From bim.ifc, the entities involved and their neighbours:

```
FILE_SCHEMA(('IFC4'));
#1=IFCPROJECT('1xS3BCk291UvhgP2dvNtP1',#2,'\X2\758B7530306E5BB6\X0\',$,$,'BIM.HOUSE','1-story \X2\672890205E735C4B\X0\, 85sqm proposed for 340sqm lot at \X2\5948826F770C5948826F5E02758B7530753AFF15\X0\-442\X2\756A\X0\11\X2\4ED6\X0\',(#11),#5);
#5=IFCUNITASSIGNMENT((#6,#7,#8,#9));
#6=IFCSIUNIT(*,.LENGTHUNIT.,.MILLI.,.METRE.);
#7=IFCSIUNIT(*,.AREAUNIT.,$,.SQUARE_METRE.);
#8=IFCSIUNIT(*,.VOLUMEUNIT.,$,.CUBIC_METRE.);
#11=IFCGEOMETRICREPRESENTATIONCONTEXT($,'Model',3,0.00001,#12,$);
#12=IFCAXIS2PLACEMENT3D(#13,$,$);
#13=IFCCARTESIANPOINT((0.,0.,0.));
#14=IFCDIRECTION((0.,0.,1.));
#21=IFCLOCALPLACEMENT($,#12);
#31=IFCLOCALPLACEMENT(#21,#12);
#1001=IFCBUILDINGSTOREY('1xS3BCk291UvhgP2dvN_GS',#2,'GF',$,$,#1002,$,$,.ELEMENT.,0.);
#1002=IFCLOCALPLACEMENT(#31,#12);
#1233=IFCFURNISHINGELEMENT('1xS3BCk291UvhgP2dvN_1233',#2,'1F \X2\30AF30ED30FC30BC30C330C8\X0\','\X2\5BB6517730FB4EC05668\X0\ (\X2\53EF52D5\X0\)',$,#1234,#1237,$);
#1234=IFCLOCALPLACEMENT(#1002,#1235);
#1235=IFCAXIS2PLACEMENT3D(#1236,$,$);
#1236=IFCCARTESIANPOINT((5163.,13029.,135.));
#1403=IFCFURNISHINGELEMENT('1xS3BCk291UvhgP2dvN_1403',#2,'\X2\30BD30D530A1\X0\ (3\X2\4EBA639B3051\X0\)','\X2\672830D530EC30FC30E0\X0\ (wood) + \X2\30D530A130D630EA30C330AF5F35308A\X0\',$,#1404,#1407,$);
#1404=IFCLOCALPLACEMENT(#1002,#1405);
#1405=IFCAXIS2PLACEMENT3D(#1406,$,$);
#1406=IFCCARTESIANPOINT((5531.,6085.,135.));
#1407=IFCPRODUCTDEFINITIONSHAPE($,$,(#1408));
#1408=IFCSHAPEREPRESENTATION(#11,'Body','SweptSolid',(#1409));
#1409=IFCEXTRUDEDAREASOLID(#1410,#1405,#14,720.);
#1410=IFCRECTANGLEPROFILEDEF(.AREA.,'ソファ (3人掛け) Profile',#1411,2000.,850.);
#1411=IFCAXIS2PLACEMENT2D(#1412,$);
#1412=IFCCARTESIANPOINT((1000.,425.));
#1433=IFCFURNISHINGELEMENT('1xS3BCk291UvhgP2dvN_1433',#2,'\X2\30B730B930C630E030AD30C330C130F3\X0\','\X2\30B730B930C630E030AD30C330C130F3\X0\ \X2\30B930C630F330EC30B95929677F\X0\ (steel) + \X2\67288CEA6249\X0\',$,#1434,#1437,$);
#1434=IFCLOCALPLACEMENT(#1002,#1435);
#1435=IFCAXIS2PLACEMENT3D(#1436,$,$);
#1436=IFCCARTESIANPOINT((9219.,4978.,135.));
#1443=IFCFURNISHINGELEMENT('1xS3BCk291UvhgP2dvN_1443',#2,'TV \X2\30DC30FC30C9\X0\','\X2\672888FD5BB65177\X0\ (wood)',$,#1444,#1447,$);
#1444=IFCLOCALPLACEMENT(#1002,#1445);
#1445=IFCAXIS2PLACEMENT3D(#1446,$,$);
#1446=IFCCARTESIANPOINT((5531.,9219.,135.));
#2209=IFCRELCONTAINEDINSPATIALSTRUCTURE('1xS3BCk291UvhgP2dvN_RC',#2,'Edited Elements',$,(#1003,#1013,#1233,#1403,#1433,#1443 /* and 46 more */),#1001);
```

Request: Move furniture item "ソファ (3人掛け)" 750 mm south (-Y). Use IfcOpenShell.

```python
import ifcopenshell
import ifcopenshell.api.geometry
import ifcopenshell.util.placement

model = ifcopenshell.open("bim.ifc")

item = model.by_guid("1xS3BCk291UvhgP2dvN_1403")
matrix = ifcopenshell.util.placement.get_local_placement(item.ObjectPlacement)
matrix[1, 3] -= 750.0
ifcopenshell.api.geometry.edit_object_placement(model, product=item, matrix=matrix, is_si=False)

print(ifcopenshell.util.placement.get_local_placement(item.ObjectPlacement).round(3) + 0.0)

model.write("bim_v2.ifc")
```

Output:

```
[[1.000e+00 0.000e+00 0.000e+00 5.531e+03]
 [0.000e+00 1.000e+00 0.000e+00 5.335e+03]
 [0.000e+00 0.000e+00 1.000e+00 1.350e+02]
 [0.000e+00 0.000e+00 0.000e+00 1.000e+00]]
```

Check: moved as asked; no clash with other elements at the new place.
